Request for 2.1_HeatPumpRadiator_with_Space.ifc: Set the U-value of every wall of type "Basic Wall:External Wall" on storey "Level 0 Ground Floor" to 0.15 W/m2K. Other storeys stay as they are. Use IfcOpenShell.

First a look at what the model holds.

```python
import ifcopenshell
import ifcopenshell.util.element

model = ifcopenshell.open("2.1_HeatPumpRadiator_with_Space.ifc")
print(model.schema)
storey = next(s for s in model.by_type("IfcBuildingStorey") if s.Name == "Level 0 Ground Floor")
walls = [e for e in ifcopenshell.util.element.get_decomposition(storey) if e.is_a("IfcWall")]
seen = {}
for e in walls:
    element_type = ifcopenshell.util.element.get_type(e)
    key = (element_type.Name if element_type != e and element_type else None, ifcopenshell.util.element.get_pset(e, "Pset_WallCommon", "ThermalTransmittance"))
    seen[key] = seen.get(key, 0) + 1
for (name, value), count in sorted(seen.items(), key=str):
    print(count, "x", name, "|", value)
```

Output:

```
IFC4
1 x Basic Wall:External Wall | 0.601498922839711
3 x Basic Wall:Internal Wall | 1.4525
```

```python
import ifcopenshell
import ifcopenshell.api.pset
import ifcopenshell.util.element

model = ifcopenshell.open("2.1_HeatPumpRadiator_with_Space.ifc")

storey = next(s for s in model.by_type("IfcBuildingStorey") if s.Name == "Level 0 Ground Floor")
walls = [e for e in ifcopenshell.util.element.get_decomposition(storey) if e.is_a("IfcWall")]

count = 0
for e in walls:
    element_type = ifcopenshell.util.element.get_type(e)
    if element_type in (None, e) or element_type.Name != "Basic Wall:External Wall":
        continue
    # add_pset returns the element's existing set when there is one.
    pset = ifcopenshell.api.pset.add_pset(model, product=e, name="Pset_WallCommon")
    ifcopenshell.api.pset.edit_pset(model, pset=pset, properties={"ThermalTransmittance": 0.15})
    count += 1

print(count, "walls updated")

model.write("2.1_HeatPumpRadiator_with_Space-out.ifc")
```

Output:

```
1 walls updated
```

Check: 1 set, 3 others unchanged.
